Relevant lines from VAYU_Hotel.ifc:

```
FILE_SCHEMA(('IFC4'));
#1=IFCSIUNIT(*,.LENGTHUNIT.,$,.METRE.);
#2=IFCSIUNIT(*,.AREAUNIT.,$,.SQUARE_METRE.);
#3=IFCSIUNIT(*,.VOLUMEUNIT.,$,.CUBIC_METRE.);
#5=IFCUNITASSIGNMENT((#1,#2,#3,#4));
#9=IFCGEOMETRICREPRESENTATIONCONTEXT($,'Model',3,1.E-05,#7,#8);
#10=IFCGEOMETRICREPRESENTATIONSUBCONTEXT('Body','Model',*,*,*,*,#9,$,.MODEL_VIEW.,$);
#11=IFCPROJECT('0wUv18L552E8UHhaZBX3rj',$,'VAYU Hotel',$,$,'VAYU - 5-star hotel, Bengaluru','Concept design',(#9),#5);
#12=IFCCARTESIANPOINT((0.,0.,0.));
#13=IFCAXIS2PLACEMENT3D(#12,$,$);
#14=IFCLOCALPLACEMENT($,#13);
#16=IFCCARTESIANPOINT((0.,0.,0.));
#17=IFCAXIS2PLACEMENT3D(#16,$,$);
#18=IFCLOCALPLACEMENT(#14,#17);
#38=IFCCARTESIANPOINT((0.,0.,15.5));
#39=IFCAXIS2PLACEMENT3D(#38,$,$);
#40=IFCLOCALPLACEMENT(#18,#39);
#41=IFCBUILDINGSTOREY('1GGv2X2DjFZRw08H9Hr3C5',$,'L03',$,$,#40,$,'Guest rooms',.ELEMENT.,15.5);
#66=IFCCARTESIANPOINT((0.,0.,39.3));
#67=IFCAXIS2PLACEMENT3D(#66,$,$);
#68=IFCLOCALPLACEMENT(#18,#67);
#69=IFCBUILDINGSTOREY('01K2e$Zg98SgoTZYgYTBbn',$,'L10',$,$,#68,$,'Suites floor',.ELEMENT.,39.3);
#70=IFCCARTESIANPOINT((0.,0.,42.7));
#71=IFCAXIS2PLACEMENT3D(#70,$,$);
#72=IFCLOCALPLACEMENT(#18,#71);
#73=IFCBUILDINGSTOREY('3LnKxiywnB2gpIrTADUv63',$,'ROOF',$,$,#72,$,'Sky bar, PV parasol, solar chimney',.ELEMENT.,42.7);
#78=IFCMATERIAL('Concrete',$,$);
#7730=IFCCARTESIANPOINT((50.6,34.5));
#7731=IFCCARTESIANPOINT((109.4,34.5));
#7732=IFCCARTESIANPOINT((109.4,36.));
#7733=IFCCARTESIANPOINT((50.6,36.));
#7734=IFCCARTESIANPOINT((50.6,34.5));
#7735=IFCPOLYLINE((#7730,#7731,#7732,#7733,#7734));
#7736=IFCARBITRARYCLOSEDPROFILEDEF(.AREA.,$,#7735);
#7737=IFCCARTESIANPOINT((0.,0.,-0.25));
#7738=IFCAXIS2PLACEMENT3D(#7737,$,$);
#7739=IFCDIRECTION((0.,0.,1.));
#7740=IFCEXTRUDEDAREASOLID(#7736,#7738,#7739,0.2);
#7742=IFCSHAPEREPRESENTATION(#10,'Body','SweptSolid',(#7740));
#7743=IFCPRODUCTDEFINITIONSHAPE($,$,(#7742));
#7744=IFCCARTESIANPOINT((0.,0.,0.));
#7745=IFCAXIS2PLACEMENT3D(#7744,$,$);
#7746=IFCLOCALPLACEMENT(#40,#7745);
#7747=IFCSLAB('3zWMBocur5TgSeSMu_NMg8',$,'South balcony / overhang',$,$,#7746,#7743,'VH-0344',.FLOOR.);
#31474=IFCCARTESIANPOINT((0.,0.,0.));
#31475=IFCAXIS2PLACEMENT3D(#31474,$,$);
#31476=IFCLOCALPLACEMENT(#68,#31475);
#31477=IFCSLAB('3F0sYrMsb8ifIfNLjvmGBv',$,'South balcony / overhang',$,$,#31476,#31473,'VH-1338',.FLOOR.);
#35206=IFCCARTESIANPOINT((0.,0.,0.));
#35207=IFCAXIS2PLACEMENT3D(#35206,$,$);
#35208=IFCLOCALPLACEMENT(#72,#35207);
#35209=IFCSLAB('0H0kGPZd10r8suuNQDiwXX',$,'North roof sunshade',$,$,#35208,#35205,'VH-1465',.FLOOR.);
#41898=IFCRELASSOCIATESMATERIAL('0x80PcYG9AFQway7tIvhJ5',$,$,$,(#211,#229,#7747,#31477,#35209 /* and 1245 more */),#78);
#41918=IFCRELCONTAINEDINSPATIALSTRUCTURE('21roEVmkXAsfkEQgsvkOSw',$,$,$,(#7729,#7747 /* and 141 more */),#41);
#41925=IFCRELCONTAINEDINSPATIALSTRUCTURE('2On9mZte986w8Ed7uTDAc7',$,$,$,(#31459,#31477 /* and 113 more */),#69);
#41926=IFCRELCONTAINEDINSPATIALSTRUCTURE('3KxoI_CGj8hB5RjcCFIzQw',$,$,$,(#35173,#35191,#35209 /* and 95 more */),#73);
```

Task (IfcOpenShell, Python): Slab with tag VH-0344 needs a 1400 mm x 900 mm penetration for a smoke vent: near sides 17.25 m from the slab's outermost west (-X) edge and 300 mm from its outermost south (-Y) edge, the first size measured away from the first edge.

```python
import numpy as np
import ifcopenshell
import ifcopenshell.api.feature
import ifcopenshell.api.geometry
import ifcopenshell.api.root
import ifcopenshell.geom
import ifcopenshell.util.placement
import ifcopenshell.util.representation
import ifcopenshell.util.shape
import ifcopenshell.util.unit

model = ifcopenshell.open("VAYU_Hotel.ifc")
unit_scale = ifcopenshell.util.unit.calculate_unit_scale(model)
settings = ifcopenshell.geom.settings()


def volume(element):
    """Net volume in cubic metres, openings subtracted."""
    shape = ifcopenshell.geom.create_shape(settings, element)
    return ifcopenshell.util.shape.get_volume(shape.geometry)


slab = model.by_guid("3zWMBocur5TgSeSMu_NMg8")
before = volume(slab)

# Extent in the slab's own axes, in metres. The edges named are its -X and -Y sides.
slab_shape = ifcopenshell.geom.create_shape(settings, slab)
vertices = ifcopenshell.util.shape.get_vertices(slab_shape.geometry)
x_min, y_min, bottom = vertices.min(axis=0)
top = vertices[:, 2].max()

opening = ifcopenshell.api.root.create_entity(model, ifc_class="IfcOpeningElement", name="Smoke vent opening", predefined_type="OPENING")
context = ifcopenshell.util.representation.get_context(model, "Model", "Body", "MODEL_VIEW")
width, depth = 1.4, 0.9
outline = [(0.0, 0.0), (width, 0.0), (width, depth), (0.0, depth), (0.0, 0.0)]
# Overshoot both faces by 50 mm so the cut is clean.
shape = ifcopenshell.api.geometry.add_slab_representation(
    model, context=context, depth=top - bottom + 0.1, polyline=outline
)
ifcopenshell.api.geometry.assign_representation(model, product=opening, representation=shape)

matrix = ifcopenshell.util.placement.get_local_placement(slab.ObjectPlacement)
matrix[:, 3] = matrix @ np.append(np.array([x_min + 17.25, y_min + 0.3, bottom - 0.05]) / unit_scale, 1.0)
ifcopenshell.api.geometry.edit_object_placement(model, product=opening, matrix=matrix, is_si=False)
ifcopenshell.api.feature.add_feature(model, feature=opening, element=slab)

after = volume(slab)

print(f"slab volume {before:.3f} -> {after:.3f} m3")

model.write("VAYU_Hotel_updated.ifc")
```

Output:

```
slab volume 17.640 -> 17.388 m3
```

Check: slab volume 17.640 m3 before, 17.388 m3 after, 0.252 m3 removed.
